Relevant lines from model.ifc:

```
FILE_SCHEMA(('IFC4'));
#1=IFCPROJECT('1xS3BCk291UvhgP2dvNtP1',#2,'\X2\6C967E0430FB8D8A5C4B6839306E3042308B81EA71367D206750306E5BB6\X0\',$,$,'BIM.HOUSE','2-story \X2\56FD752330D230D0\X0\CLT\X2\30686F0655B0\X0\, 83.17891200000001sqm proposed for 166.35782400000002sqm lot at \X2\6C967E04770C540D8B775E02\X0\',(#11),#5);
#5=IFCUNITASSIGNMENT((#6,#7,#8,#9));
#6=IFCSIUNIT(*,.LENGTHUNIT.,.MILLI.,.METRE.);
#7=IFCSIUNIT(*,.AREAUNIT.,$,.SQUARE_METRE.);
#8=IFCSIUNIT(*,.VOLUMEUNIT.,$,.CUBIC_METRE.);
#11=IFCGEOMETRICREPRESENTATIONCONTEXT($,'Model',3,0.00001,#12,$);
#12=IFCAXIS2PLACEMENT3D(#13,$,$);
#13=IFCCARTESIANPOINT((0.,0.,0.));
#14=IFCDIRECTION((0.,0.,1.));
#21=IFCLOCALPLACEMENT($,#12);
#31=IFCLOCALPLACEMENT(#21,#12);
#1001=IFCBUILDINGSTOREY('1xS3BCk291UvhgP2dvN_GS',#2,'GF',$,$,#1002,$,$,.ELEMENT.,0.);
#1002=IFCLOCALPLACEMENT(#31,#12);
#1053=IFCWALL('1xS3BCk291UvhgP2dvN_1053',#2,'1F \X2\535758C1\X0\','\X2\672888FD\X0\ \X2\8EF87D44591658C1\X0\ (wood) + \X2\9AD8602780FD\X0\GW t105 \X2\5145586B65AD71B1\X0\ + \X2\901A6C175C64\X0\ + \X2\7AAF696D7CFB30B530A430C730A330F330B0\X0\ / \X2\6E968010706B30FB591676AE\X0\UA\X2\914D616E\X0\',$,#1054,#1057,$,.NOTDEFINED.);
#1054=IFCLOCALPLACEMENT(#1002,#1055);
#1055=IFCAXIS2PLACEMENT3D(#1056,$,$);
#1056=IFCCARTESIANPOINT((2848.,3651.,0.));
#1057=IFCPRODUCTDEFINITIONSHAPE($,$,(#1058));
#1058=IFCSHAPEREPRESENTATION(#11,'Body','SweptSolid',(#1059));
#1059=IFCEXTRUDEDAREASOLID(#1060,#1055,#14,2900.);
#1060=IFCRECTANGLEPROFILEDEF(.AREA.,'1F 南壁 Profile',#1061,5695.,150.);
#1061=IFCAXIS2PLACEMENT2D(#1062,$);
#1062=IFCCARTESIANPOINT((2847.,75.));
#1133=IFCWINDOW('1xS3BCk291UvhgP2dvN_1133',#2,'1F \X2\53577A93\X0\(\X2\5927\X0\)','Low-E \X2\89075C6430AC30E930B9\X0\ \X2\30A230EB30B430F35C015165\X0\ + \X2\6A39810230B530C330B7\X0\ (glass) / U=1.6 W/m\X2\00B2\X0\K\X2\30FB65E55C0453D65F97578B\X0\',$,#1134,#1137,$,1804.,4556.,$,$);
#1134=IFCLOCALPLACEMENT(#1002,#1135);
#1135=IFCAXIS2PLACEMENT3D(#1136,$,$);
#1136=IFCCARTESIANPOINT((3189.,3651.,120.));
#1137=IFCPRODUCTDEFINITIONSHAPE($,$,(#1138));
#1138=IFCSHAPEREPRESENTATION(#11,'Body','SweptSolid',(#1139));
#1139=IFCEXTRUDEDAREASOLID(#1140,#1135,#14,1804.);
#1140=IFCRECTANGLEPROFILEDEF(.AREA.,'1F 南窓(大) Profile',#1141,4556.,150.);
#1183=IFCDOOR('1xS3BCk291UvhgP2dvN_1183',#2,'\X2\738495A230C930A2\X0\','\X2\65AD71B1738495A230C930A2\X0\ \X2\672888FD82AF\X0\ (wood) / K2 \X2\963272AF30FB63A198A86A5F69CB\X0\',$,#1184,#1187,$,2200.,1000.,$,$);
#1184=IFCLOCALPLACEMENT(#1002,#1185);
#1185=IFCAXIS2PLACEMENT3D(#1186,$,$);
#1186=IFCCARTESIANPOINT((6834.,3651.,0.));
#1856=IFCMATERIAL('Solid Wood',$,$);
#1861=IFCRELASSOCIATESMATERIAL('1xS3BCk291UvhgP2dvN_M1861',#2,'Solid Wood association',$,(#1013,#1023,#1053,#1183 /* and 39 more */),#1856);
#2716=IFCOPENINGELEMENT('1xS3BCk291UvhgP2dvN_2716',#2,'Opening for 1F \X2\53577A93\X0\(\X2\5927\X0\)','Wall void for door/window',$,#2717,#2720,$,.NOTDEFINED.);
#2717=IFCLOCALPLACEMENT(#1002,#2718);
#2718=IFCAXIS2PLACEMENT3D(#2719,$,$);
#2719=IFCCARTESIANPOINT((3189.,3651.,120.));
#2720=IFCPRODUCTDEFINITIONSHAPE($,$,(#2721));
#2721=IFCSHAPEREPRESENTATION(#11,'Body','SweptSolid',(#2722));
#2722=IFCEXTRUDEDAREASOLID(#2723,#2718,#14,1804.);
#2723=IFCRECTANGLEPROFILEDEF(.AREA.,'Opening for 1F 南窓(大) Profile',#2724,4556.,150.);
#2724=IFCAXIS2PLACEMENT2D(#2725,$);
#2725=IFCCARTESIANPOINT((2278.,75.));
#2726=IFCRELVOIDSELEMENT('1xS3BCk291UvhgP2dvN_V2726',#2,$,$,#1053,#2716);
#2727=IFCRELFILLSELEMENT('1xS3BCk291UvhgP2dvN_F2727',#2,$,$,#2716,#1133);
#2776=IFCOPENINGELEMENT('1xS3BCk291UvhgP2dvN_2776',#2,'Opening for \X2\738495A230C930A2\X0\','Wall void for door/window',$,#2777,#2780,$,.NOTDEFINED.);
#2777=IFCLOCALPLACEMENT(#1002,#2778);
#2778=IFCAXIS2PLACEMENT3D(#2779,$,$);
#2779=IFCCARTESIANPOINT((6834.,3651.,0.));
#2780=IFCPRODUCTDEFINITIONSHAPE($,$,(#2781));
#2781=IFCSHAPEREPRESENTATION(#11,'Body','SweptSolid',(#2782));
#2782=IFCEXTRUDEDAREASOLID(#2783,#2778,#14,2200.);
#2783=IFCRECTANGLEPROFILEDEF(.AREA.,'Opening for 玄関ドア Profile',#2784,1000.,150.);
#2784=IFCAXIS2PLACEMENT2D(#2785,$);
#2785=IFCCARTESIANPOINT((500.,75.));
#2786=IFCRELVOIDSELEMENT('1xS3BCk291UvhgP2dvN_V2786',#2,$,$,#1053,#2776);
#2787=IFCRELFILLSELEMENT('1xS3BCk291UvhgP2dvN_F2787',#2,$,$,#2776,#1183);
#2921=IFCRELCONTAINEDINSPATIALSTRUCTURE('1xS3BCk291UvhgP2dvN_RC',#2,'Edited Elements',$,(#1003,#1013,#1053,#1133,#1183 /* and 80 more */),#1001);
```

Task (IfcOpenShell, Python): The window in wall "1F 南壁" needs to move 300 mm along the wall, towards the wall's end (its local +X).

```python
import ifcopenshell
import ifcopenshell.api.geometry
import ifcopenshell.util.placement
import ifcopenshell.util.unit

model = ifcopenshell.open("model.ifc")
unit_scale = ifcopenshell.util.unit.calculate_unit_scale(model)

window = model.by_guid("1xS3BCk291UvhgP2dvN_1133")
opening = window.FillsVoids[0].RelatingOpeningElement
wall = opening.VoidsElements[0].RelatingBuildingElement

wall_matrix = ifcopenshell.util.placement.get_local_placement(wall.ObjectPlacement)
shift = wall_matrix[:3, 0] * 0.3 / unit_scale
before = ifcopenshell.util.placement.get_local_placement(window.ObjectPlacement)[:3, 3].copy()

# The window is not placed relative to its opening, so move both.
for product in (opening, window):
    matrix = ifcopenshell.util.placement.get_local_placement(product.ObjectPlacement)
    matrix[:3, 3] += shift
    ifcopenshell.api.geometry.edit_object_placement(model, product=product, matrix=matrix, is_si=False)

after = ifcopenshell.util.placement.get_local_placement(window.ObjectPlacement)[:3, 3]
print("window moved by", (after - before).round(3) + 0.0)

model.write("model-out.ifc")
```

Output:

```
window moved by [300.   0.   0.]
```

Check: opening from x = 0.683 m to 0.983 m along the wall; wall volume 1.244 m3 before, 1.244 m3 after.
